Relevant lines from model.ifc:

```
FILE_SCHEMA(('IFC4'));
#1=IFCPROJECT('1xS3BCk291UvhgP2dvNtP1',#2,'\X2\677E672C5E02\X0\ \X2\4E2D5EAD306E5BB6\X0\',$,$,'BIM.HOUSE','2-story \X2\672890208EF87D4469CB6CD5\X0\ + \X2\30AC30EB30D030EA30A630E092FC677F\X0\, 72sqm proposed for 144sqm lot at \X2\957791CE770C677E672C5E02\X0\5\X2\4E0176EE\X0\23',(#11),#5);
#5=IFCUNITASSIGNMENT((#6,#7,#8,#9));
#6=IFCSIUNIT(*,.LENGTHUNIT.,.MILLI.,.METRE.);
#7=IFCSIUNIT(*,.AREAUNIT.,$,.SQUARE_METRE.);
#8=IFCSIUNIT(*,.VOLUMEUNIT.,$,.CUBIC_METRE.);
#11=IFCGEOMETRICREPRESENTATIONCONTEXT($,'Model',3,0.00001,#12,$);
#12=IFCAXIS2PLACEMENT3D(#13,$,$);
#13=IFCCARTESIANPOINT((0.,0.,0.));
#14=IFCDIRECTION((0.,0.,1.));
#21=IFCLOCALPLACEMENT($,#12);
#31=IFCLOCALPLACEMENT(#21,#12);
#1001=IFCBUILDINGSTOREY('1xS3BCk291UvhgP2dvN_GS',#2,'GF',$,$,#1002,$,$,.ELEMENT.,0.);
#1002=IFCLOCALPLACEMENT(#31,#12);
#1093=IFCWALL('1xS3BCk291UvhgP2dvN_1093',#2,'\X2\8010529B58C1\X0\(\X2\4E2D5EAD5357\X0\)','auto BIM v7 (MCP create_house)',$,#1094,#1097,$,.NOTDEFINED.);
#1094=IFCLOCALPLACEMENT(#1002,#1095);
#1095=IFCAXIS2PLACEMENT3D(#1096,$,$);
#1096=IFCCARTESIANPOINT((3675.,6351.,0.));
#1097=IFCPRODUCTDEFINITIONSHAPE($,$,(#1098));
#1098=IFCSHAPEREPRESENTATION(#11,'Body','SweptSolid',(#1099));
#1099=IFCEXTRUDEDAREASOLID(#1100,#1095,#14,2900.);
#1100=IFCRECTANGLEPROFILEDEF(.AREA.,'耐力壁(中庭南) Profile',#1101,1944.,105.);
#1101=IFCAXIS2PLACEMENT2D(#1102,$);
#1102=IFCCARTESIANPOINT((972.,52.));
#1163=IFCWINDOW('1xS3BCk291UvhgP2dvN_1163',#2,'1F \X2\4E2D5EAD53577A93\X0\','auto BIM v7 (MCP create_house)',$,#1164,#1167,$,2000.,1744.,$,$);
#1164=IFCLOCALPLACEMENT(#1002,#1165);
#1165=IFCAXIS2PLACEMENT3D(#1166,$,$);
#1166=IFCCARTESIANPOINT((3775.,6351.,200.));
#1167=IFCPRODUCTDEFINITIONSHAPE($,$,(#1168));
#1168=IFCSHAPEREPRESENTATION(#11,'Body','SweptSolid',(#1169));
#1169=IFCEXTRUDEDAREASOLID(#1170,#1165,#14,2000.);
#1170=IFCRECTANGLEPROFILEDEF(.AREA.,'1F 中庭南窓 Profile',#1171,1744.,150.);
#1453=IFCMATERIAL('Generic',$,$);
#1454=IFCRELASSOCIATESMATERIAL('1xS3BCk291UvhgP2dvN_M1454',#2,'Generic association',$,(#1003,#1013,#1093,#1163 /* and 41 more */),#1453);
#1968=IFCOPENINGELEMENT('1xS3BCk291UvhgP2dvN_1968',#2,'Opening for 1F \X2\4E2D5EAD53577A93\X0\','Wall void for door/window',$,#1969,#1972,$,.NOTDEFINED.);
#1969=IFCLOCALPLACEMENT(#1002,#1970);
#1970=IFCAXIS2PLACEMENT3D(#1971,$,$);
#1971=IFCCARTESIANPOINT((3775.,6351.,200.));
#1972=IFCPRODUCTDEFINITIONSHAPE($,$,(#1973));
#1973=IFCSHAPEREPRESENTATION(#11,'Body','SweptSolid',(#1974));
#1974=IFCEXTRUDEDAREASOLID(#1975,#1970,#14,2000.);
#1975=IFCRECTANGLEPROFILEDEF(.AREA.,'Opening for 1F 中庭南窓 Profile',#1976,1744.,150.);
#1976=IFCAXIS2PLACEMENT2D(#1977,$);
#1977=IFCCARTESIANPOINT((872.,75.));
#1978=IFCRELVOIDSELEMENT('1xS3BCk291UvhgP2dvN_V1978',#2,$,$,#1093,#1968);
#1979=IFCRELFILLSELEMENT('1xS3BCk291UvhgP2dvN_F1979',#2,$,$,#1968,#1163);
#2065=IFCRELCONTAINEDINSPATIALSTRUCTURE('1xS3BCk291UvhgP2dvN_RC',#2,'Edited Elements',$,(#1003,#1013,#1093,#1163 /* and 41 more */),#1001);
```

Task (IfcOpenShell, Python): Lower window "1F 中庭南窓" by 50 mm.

```python
import numpy as np
import ifcopenshell
import ifcopenshell.api.geometry
import ifcopenshell.util.placement
import ifcopenshell.util.unit

model = ifcopenshell.open("model.ifc")
unit_scale = ifcopenshell.util.unit.calculate_unit_scale(model)

window = model.by_guid("1xS3BCk291UvhgP2dvN_1163")
opening = window.FillsVoids[0].RelatingOpeningElement
dz = -0.05 / unit_scale

shift = np.array([0.0, 0.0, dz])
# The window is not placed relative to its opening, so move both.
for product in (opening, window):
    matrix = ifcopenshell.util.placement.get_local_placement(product.ObjectPlacement)
    matrix[:3, 3] += shift
    ifcopenshell.api.geometry.edit_object_placement(model, product=product, matrix=matrix, is_si=False)

print(f"moved by {dz * unit_scale:+.3f} m")

model.write("model_edited.ifc")
```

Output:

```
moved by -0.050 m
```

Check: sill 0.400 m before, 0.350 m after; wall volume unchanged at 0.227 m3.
